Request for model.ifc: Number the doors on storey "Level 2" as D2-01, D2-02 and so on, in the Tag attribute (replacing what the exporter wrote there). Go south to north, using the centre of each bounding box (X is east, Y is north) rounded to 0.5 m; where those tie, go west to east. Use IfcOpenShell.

First a look at what the model holds.

```python
import ifcopenshell
import ifcopenshell.util.element
import ifcopenshell.util.placement

model = ifcopenshell.open("model.ifc")
print(model.schema)
storey = next(s for s in model.by_type("IfcBuildingStorey") if s.Name == "Level 2")
doors = [e for e in ifcopenshell.util.element.get_decomposition(storey) if e.is_a("IfcDoor")]
for e in sorted(doors, key=lambda e: e.id()):
    origin = ifcopenshell.util.placement.get_local_placement(e.ObjectPlacement)[:3, 3]
    print(e.id(), e.Tag, e.Name, origin.round(2) + 0.0, sep=" | ")
```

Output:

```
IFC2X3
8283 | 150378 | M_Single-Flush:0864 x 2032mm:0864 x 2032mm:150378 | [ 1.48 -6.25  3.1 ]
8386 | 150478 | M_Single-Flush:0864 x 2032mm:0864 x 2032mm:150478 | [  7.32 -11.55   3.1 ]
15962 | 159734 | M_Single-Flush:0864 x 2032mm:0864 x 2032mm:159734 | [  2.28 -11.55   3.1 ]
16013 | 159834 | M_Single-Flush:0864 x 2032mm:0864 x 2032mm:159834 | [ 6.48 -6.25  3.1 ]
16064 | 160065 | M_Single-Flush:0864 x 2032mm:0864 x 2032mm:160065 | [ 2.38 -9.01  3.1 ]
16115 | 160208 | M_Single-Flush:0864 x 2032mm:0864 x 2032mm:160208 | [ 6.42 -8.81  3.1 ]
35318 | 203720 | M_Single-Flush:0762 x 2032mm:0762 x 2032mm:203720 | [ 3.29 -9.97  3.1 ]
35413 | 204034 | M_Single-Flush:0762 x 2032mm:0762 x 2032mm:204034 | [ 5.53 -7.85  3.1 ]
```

```python
import ifcopenshell
import ifcopenshell.geom
import ifcopenshell.util.element
import ifcopenshell.util.shape

model = ifcopenshell.open("model.ifc")
settings = ifcopenshell.geom.settings()
settings.set("use-world-coords", True)


def centre(element):
    shape = ifcopenshell.geom.create_shape(settings, element)
    return ifcopenshell.util.shape.get_bbox_centroid(shape.geometry)


storey = next(s for s in model.by_type("IfcBuildingStorey") if s.Name == "Level 2")
doors = [e for e in ifcopenshell.util.element.get_decomposition(storey) if e.is_a("IfcDoor")]

# Insertion points can sit at a corner or the storey origin, so sort by the geometry (in metres).
centres = {e: centre(e) for e in doors}
doors.sort(key=lambda e: (round(centres[e][1] / 0.5), centres[e][0]))

for i, e in enumerate(doors, start=1):
    number = f"D2-{i:02d}"
    e.Tag = number
    print(e.id(), number)

model.write("model-out.ifc")
```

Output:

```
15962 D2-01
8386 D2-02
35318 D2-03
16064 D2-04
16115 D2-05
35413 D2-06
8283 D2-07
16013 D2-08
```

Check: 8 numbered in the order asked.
